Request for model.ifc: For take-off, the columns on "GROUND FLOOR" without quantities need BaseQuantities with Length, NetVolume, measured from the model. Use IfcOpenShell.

First a look at what the model holds.

```python
import ifcopenshell
import ifcopenshell.util.element
import ifcopenshell.util.unit

model = ifcopenshell.open("model.ifc")
print(model.schema)
for unit_type in ("LENGTHUNIT", "AREAUNIT", "VOLUMEUNIT"):
    print(unit_type, ifcopenshell.util.unit.calculate_unit_scale(model, unit_type))
storey = next(s for s in model.by_type("IfcBuildingStorey") if s.Name == "GROUND FLOOR")
columns = [e for e in ifcopenshell.util.element.get_decomposition(storey) if e.is_a("IfcColumn")]
for e in sorted(columns, key=lambda e: e.id()):
    print(e.id(), e.is_a(), e.Name, list(ifcopenshell.util.element.get_psets(e, qtos_only=True)), sep=" | ")
```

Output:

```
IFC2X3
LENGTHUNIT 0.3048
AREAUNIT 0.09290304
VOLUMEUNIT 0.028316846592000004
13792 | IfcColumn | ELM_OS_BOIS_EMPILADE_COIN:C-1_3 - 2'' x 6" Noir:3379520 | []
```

```python
import ifcopenshell
import ifcopenshell.api.pset
import ifcopenshell.geom
import ifcopenshell.util.element
import ifcopenshell.util.shape
import ifcopenshell.util.unit

model = ifcopenshell.open("model.ifc")
unit_scale = ifcopenshell.util.unit.calculate_unit_scale(model)
volume_scale = ifcopenshell.util.unit.calculate_unit_scale(model, "VOLUMEUNIT")
settings = ifcopenshell.geom.settings()

storey = next(s for s in model.by_type("IfcBuildingStorey") if s.Name == "GROUND FLOOR")
columns = [e for e in ifcopenshell.util.element.get_decomposition(storey) if e.is_a("IfcColumn")]

for e in sorted(columns, key=lambda e: e.id()):
    if ifcopenshell.util.element.get_psets(e, qtos_only=True, should_inherit=False):
        continue
    # Geometry comes back in metres, in the element's own axes.
    shape = ifcopenshell.geom.create_shape(settings, e)
    values = {
        "Length": ifcopenshell.util.shape.get_z(shape.geometry) / unit_scale,
        "NetVolume": ifcopenshell.util.shape.get_volume(shape.geometry) / volume_scale,
    }
    qto = ifcopenshell.api.pset.add_qto(model, product=e, name="BaseQuantities")
    ifcopenshell.api.pset.edit_qto(model, qto=qto, properties=values)
    print(e.id(), {k: round(v, 3) for k, v in values.items()})

model.write("model_edited.ifc")
```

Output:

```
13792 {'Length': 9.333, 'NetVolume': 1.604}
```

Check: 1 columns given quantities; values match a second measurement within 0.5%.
